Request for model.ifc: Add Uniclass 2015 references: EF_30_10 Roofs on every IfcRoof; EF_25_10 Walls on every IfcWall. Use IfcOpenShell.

First a look at what the model holds.

```python
import ifcopenshell

model = ifcopenshell.open("model.ifc")
print(model.schema)
print("classifications:", [c.Name for c in model.by_type("IfcClassification")])
for ifc_class in ("IfcDoor", "IfcRoof", "IfcStair", "IfcWall", "IfcWindow"):
    print(ifc_class, len(model.by_type(ifc_class)))
```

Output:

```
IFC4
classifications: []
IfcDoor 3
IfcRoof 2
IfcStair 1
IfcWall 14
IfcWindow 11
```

```python
import ifcopenshell
import ifcopenshell.api.classification

model = ifcopenshell.open("model.ifc")

system = ifcopenshell.api.classification.add_classification(model, classification="Uniclass 2015")

codes = {
    "IfcRoof": ("EF_30_10", "Roofs"),
    "IfcWall": ("EF_25_10", "Walls"),
}
for ifc_class, (code, name) in codes.items():
    products = model.by_type(ifc_class)
    ifcopenshell.api.classification.add_reference(
        model, products=products, classification=system, identification=code, name=name
    )
    print(code, len(products))

model.write("model_edited.ifc")
```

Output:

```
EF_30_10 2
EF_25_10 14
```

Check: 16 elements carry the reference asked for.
